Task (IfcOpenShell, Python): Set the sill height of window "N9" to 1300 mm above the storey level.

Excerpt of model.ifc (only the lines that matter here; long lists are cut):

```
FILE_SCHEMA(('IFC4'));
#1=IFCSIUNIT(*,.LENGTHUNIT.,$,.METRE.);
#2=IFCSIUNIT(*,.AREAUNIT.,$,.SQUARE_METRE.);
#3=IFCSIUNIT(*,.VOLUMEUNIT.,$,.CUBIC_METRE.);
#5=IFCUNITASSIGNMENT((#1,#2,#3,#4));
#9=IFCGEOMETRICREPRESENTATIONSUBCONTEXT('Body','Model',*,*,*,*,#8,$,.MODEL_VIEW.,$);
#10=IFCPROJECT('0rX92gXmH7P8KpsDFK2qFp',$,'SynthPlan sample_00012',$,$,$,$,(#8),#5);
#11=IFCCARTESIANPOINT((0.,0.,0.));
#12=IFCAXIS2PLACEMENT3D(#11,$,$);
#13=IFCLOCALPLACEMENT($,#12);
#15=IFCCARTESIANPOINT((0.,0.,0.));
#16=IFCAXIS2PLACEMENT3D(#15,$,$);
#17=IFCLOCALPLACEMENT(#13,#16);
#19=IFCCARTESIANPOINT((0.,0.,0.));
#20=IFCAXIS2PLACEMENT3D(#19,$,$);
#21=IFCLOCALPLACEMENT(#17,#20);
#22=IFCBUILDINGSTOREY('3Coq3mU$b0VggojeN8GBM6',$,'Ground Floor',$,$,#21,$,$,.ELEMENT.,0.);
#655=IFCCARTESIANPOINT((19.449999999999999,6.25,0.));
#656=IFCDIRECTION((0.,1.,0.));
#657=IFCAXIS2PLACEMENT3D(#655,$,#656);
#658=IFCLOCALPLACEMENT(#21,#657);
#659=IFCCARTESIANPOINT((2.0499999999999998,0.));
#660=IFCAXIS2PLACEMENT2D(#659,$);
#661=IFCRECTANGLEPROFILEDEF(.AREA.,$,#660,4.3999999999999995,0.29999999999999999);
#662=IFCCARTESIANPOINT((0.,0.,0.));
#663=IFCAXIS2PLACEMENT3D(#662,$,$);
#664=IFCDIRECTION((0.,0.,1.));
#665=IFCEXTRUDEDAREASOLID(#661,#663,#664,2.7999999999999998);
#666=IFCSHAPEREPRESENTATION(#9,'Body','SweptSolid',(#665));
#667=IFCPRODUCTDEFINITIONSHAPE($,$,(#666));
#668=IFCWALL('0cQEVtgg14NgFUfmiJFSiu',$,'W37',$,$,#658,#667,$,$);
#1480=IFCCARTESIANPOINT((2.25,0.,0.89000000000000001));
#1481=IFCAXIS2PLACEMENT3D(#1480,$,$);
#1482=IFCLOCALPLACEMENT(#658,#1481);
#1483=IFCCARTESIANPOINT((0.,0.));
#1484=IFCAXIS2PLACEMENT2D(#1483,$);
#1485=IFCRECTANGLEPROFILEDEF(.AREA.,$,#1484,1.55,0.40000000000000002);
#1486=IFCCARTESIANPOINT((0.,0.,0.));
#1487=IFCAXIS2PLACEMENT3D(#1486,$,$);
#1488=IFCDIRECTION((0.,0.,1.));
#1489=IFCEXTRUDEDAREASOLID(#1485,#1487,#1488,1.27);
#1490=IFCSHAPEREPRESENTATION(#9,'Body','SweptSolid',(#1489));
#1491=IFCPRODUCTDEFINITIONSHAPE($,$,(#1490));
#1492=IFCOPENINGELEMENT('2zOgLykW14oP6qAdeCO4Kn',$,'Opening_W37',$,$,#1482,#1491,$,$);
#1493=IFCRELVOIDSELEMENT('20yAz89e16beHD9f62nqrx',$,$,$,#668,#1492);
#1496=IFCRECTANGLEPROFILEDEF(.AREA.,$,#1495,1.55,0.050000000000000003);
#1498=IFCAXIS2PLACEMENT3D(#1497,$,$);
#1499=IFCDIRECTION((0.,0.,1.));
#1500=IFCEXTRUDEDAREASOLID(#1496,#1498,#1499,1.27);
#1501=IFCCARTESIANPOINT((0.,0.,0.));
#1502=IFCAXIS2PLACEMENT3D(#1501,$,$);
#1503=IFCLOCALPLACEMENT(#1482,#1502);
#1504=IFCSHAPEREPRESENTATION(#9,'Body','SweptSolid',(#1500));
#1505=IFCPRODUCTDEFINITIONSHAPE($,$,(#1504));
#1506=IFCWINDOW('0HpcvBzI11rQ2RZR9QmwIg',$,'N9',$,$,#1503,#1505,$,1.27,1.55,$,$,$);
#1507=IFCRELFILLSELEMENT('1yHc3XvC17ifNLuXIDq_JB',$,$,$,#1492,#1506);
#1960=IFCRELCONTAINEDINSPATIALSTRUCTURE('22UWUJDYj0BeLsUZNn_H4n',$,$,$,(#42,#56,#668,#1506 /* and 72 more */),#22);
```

```python
import numpy as np
import ifcopenshell
import ifcopenshell.api.geometry
import ifcopenshell.geom
import ifcopenshell.util.element
import ifcopenshell.util.placement
import ifcopenshell.util.shape
import ifcopenshell.util.unit

model = ifcopenshell.open("model.ifc")
unit_scale = ifcopenshell.util.unit.calculate_unit_scale(model)

window = model.by_id(1506)
opening = window.FillsVoids[0].RelatingOpeningElement
storey = ifcopenshell.util.element.get_container(window, ifc_class="IfcBuildingStorey")
level = ifcopenshell.util.placement.get_local_placement(storey.ObjectPlacement)[2, 3]

# The opening's origin need not be at the sill, so measure its lowest point.
shape = ifcopenshell.geom.create_shape(ifcopenshell.geom.settings(), opening)
bottom = ifcopenshell.util.shape.get_shape_bottom_elevation(shape, shape.geometry) / unit_scale
dz = level + 1.3 / unit_scale - bottom

shift = np.array([0.0, 0.0, dz])
# The window is placed relative to its opening, so it follows when the opening moves.
matrix = ifcopenshell.util.placement.get_local_placement(opening.ObjectPlacement)
matrix[:3, 3] += shift
ifcopenshell.api.geometry.edit_object_placement(
    model, product=opening, matrix=matrix, is_si=False, should_transform_children=True
)

print(f"moved by {dz * unit_scale:+.3f} m")

model.write("model_edited.ifc")
```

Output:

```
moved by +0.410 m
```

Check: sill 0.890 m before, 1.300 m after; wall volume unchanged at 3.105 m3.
